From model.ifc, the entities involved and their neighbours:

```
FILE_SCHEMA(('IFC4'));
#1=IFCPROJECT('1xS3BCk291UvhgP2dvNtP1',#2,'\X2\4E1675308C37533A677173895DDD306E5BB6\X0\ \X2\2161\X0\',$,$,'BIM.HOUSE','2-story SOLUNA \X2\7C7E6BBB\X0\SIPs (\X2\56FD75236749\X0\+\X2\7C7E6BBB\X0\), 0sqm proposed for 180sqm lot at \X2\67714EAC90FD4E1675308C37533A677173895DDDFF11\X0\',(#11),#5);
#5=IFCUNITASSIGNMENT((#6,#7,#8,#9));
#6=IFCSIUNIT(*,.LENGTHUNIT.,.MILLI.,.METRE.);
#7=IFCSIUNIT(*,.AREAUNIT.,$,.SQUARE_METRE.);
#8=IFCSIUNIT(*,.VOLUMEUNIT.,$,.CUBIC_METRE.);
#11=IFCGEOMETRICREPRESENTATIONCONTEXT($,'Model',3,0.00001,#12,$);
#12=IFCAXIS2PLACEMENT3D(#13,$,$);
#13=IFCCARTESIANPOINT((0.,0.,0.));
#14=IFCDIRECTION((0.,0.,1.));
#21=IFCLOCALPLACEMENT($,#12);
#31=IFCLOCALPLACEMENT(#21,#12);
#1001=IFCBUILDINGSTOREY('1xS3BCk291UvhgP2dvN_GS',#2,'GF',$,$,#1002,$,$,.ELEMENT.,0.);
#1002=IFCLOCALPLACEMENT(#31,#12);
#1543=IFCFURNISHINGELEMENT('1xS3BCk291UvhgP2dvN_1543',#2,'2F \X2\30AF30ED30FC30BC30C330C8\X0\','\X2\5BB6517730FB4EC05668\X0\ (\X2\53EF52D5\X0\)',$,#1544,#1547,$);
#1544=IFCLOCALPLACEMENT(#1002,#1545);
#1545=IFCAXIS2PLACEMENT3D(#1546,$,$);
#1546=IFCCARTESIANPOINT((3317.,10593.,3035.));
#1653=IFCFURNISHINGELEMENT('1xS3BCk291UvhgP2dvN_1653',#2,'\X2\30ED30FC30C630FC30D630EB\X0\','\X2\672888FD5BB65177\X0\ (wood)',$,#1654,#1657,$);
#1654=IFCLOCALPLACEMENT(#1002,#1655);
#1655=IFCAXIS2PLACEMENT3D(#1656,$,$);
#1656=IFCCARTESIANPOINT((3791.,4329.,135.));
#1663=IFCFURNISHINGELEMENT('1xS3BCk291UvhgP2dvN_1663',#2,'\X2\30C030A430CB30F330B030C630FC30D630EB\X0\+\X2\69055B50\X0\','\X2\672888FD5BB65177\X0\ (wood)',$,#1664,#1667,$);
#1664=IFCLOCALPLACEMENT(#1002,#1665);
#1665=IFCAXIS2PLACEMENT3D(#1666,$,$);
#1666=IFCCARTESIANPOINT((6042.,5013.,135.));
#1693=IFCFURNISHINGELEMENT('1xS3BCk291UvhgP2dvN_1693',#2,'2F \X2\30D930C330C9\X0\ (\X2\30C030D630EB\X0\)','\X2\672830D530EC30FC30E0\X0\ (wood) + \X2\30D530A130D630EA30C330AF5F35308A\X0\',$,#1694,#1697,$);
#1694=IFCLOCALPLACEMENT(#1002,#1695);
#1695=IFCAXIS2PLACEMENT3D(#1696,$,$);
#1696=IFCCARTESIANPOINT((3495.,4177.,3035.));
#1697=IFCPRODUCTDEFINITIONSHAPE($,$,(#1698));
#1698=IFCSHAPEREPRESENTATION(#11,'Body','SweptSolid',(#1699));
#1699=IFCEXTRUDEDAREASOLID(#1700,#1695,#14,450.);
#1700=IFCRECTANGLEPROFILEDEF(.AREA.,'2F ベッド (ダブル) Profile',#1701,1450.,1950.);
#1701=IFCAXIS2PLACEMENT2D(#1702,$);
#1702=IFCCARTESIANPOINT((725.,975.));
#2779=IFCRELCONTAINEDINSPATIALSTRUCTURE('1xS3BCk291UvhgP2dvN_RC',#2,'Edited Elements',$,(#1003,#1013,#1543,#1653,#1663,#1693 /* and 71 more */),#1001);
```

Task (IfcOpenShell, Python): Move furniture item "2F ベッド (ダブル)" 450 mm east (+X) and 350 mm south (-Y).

```python
import ifcopenshell
import ifcopenshell.api.geometry
import ifcopenshell.util.placement
import ifcopenshell.util.unit

model = ifcopenshell.open("model.ifc")
unit_scale = ifcopenshell.util.unit.calculate_unit_scale(model)

item = model.by_id(1693)
matrix = ifcopenshell.util.placement.get_local_placement(item.ObjectPlacement)
matrix[0, 3] += 0.45 / unit_scale
matrix[1, 3] -= 0.35 / unit_scale
ifcopenshell.api.geometry.edit_object_placement(model, product=item, matrix=matrix, is_si=False)

print(ifcopenshell.util.placement.get_local_placement(item.ObjectPlacement).round(3) + 0.0)

model.write("model_v2.ifc")
```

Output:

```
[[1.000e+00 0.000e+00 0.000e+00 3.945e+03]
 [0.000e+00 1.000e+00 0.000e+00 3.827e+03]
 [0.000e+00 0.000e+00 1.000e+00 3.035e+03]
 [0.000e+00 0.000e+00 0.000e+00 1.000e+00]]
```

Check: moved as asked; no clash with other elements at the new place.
